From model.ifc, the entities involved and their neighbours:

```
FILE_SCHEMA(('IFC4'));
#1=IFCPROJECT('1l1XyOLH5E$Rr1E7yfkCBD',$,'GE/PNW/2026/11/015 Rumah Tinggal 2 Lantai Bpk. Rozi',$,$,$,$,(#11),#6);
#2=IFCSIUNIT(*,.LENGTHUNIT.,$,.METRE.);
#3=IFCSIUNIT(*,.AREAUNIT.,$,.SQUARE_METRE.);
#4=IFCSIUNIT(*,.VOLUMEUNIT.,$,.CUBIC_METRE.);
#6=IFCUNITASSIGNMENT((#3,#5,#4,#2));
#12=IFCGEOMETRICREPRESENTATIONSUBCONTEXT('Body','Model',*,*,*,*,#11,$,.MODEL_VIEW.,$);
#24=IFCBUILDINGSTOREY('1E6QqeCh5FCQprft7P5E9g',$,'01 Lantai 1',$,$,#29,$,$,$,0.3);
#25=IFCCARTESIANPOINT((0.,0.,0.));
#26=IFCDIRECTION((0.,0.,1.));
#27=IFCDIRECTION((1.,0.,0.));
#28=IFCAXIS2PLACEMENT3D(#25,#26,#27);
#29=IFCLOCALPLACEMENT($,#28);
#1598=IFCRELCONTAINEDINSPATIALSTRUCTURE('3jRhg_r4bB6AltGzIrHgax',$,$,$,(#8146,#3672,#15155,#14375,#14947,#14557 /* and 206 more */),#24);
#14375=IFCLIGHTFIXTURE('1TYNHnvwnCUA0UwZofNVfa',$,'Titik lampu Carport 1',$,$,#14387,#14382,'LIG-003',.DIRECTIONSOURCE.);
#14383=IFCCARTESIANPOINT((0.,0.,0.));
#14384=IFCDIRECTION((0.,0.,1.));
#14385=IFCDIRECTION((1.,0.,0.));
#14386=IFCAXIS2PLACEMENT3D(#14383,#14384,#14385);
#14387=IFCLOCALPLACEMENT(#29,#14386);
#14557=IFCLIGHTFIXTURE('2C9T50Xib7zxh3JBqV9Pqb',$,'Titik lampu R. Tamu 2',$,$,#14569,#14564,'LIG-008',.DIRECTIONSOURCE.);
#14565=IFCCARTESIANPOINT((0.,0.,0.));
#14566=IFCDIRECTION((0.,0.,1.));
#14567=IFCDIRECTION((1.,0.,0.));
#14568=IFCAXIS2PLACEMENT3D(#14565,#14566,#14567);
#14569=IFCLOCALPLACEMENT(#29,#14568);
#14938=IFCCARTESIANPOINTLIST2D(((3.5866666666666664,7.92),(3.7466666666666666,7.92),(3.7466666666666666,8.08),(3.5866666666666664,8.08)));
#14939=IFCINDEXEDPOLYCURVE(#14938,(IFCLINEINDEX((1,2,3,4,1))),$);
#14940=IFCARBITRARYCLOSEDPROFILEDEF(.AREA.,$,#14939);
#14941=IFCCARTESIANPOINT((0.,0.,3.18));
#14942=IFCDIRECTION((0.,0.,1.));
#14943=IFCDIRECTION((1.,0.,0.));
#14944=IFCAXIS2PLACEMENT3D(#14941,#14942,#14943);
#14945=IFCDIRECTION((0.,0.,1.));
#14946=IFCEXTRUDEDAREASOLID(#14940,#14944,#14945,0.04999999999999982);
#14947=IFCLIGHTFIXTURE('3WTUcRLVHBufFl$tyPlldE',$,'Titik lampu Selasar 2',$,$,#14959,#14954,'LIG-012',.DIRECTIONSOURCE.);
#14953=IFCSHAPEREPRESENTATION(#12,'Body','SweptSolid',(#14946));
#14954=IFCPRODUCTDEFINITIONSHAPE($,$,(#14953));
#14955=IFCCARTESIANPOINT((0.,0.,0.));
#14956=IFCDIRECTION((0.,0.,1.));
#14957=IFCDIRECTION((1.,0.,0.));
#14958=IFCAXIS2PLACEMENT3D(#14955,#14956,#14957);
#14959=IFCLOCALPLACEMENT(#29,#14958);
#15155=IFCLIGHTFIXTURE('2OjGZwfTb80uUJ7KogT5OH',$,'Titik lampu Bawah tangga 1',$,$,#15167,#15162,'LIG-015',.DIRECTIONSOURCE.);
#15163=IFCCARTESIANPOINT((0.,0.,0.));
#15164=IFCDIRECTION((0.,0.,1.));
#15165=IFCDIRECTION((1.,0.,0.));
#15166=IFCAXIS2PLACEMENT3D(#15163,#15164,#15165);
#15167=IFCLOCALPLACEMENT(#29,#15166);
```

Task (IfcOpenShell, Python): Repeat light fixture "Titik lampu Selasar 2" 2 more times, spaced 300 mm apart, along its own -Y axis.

```python
import ifcopenshell
import ifcopenshell.api.geometry
import ifcopenshell.api.root
import ifcopenshell.util.element
import ifcopenshell.util.placement
import ifcopenshell.util.unit

model = ifcopenshell.open("model.ifc")
unit_scale = ifcopenshell.util.unit.calculate_unit_scale(model)

source = model.by_guid("3WTUcRLVHBufFl$tyPlldE")
base = ifcopenshell.util.placement.get_local_placement(source.ObjectPlacement)
step = -base[:3, 1] * 0.3 / unit_scale

for i in range(1, 3):
    copy = ifcopenshell.api.root.copy_class(model, product=source)
    copy.Representation = ifcopenshell.util.element.copy_deep(
        model, source.Representation, exclude=["IfcGeometricRepresentationContext", "IfcRepresentationMap"]
    )
    copy.Tag = None
    matrix = base.copy()
    matrix[:3, 3] += i * step
    print("added at", matrix[:3, 3].round(3) + 0.0)
    ifcopenshell.api.geometry.edit_object_placement(model, product=copy, matrix=matrix, is_si=False)

model.write("model_rev.ifc")
```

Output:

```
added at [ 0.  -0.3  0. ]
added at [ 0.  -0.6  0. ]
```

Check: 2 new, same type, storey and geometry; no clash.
